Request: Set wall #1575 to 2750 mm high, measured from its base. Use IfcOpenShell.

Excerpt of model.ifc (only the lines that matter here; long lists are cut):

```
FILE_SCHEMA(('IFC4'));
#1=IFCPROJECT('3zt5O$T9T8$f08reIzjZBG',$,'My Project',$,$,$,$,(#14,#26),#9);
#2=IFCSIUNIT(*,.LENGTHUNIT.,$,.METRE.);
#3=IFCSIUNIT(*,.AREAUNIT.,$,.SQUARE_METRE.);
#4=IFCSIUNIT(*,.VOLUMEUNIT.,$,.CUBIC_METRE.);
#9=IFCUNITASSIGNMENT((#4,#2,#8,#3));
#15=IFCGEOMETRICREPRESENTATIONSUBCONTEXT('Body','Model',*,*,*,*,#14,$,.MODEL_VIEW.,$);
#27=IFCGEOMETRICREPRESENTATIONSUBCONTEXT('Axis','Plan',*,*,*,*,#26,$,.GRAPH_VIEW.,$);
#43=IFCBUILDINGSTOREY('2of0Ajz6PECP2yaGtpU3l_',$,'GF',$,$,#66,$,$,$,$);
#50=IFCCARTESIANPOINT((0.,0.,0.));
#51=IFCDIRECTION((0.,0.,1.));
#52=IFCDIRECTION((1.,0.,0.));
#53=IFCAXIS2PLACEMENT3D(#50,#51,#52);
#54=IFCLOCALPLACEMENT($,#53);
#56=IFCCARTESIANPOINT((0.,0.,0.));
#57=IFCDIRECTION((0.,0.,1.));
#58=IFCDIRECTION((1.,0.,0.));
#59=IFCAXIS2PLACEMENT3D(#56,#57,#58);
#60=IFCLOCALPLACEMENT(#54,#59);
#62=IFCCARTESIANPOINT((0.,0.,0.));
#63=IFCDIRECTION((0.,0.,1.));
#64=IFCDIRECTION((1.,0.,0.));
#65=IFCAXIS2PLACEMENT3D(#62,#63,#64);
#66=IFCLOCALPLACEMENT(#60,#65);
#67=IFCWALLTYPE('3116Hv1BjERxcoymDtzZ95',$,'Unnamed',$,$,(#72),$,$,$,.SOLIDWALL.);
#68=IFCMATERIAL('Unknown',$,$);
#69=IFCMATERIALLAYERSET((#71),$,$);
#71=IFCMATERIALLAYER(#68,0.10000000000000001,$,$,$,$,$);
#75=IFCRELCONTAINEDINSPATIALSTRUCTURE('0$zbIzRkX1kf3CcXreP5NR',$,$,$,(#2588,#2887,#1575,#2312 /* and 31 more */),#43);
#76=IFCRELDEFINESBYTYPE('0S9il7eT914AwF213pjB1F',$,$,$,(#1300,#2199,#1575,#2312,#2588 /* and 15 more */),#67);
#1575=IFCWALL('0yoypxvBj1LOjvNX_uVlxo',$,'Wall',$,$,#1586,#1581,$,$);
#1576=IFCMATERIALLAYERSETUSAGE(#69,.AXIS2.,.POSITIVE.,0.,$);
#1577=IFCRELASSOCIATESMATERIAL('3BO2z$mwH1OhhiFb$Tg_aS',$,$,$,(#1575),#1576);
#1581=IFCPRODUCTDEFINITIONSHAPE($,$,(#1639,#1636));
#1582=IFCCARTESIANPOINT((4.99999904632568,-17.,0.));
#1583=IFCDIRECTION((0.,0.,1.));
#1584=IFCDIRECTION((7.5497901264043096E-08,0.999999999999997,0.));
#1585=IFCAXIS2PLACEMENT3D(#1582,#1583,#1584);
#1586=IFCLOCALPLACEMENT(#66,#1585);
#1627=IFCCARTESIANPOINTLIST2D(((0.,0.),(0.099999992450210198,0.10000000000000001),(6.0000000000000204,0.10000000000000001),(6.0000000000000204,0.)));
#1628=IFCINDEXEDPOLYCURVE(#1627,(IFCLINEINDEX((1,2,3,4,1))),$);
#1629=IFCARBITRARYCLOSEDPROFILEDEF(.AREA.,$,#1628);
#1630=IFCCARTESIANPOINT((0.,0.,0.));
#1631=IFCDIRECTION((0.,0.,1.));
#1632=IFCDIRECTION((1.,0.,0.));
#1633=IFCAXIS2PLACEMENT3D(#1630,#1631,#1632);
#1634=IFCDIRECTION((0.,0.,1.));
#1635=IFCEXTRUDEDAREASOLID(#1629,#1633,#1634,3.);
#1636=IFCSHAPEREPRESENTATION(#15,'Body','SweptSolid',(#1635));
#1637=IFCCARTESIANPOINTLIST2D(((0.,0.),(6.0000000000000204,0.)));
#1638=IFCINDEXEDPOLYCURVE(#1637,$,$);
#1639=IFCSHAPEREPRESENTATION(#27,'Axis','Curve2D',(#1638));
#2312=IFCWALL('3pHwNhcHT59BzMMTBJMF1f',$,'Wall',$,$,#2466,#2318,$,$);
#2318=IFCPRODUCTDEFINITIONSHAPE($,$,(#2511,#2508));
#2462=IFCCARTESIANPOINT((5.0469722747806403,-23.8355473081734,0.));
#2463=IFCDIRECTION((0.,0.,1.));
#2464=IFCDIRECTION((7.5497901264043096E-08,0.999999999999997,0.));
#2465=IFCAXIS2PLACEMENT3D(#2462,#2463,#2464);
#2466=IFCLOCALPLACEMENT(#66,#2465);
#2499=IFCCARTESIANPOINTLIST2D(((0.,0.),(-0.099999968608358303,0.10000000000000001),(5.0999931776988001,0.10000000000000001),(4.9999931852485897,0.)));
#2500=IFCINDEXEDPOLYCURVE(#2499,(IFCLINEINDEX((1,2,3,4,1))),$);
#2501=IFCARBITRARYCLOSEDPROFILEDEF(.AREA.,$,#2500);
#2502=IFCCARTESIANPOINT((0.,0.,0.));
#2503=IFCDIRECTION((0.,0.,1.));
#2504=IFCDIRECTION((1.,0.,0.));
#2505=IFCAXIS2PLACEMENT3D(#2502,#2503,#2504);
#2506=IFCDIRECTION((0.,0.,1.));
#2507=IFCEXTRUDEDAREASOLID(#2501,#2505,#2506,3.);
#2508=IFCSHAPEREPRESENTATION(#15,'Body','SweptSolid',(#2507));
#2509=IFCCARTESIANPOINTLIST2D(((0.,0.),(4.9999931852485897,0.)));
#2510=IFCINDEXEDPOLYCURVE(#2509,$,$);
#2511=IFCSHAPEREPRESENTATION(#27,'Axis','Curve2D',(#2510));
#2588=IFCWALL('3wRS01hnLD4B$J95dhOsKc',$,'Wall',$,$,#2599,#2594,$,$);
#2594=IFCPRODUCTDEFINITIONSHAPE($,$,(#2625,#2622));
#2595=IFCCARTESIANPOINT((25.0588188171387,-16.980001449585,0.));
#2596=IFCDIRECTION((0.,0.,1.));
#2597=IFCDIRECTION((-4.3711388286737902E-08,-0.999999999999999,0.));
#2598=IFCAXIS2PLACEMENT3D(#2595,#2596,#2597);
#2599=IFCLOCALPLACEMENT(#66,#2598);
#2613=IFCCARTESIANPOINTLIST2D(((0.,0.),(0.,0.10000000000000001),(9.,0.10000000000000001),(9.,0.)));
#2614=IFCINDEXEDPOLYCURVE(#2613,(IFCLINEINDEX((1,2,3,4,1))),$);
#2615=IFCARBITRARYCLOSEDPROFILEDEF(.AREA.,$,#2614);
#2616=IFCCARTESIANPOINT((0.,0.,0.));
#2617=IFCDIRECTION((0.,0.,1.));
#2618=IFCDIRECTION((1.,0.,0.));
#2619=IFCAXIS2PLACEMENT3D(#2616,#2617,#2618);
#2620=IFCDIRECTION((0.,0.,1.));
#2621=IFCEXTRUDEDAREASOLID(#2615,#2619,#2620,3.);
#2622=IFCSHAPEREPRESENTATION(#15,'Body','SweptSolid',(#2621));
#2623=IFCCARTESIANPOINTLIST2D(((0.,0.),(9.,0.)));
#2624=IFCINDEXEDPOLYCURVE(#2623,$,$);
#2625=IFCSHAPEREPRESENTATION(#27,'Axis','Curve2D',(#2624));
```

```python
import ifcopenshell
import ifcopenshell.geom
import ifcopenshell.util.representation
import ifcopenshell.util.shape
import ifcopenshell.util.unit

model = ifcopenshell.open("model.ifc")
unit_scale = ifcopenshell.util.unit.calculate_unit_scale(model)
settings = ifcopenshell.geom.settings()


def volume(element):
    """Net volume in cubic metres, openings subtracted."""
    shape = ifcopenshell.geom.create_shape(settings, element)
    return ifcopenshell.util.shape.get_volume(shape.geometry)


wall = model.by_guid("0yoypxvBj1LOjvNX_uVlxo")
before = volume(wall)

body = ifcopenshell.util.representation.get_representation(wall, "Model", "Body")
solid = body.Items[0]
old_height = solid.Depth
solid.Depth = 2.75 / unit_scale
after = volume(wall)

print(f"height {old_height:g} -> {solid.Depth:g}, volume {before:.3f} -> {after:.3f} m3")

model.write("model_rev.ifc")
```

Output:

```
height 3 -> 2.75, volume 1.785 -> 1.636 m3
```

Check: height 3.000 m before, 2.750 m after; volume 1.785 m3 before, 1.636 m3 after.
